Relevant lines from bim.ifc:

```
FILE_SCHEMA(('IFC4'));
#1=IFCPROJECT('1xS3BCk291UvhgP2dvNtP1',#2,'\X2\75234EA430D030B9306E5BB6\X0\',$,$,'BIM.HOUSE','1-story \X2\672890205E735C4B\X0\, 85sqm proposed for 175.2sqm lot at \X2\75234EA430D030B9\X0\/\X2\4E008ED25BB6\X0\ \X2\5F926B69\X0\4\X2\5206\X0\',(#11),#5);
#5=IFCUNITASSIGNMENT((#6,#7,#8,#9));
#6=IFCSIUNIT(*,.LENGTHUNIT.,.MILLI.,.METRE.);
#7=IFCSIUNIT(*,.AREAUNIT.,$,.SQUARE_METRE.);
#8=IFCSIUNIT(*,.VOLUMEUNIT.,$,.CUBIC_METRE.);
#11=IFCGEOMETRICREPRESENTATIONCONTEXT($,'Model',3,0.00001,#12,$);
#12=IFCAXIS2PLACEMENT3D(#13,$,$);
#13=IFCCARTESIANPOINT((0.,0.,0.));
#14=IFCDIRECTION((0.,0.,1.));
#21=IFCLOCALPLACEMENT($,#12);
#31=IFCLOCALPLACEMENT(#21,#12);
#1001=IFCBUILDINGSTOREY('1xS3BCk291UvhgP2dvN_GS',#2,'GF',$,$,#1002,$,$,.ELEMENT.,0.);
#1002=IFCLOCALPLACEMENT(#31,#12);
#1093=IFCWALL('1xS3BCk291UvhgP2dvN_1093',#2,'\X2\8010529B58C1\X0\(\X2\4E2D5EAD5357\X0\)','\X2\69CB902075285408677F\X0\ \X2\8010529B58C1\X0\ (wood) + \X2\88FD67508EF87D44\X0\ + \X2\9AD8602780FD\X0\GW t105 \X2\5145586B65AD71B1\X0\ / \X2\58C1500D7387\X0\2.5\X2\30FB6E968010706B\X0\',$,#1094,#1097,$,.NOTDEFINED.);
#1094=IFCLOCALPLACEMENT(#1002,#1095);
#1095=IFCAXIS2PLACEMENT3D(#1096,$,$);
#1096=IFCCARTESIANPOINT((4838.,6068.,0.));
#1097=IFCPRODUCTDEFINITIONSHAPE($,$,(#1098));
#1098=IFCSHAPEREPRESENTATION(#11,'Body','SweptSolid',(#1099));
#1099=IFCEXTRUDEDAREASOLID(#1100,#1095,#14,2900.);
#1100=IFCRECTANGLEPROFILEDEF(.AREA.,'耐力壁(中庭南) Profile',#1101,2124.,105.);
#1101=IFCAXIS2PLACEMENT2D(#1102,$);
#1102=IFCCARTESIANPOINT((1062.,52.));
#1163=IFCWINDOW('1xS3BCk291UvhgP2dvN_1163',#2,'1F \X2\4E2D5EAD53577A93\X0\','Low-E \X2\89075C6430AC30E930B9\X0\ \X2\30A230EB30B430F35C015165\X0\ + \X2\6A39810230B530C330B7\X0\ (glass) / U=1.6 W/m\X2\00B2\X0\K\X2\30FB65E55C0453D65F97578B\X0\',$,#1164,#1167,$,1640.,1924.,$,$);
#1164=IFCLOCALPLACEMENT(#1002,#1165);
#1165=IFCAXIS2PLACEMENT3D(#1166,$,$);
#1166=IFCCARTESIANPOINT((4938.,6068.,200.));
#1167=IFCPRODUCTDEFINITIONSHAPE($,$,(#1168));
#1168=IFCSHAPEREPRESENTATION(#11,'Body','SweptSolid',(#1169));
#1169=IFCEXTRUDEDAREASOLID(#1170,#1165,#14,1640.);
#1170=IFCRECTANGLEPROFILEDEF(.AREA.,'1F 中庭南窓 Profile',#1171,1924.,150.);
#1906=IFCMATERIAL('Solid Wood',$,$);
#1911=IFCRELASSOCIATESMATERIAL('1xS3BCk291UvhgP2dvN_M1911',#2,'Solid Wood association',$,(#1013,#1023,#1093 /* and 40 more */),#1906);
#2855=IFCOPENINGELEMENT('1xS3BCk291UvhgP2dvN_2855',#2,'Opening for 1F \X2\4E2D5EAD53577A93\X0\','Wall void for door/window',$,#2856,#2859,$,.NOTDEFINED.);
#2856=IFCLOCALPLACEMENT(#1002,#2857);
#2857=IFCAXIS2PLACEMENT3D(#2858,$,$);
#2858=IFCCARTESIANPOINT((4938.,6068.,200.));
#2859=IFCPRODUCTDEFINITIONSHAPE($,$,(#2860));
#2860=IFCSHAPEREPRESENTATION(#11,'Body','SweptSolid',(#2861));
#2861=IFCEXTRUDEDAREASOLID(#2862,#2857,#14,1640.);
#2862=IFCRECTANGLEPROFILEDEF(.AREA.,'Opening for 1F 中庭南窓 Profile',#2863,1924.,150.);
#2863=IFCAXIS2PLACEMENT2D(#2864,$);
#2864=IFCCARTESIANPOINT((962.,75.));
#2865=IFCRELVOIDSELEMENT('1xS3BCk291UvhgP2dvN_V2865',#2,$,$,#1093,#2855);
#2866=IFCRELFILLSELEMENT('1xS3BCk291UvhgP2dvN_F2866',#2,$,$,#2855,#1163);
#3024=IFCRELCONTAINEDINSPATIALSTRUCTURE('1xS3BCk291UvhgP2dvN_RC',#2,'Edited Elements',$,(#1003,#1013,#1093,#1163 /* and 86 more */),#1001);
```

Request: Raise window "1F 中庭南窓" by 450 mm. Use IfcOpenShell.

```python
import numpy as np
import ifcopenshell
import ifcopenshell.api.geometry
import ifcopenshell.util.placement
import ifcopenshell.util.unit

model = ifcopenshell.open("bim.ifc")
unit_scale = ifcopenshell.util.unit.calculate_unit_scale(model)

window = model.by_guid("1xS3BCk291UvhgP2dvN_1163")
opening = window.FillsVoids[0].RelatingOpeningElement
dz = 450.0

shift = np.array([0.0, 0.0, dz])
# The window is not placed relative to its opening, so move both.
for product in (opening, window):
    matrix = ifcopenshell.util.placement.get_local_placement(product.ObjectPlacement)
    matrix[:3, 3] += shift
    ifcopenshell.api.geometry.edit_object_placement(model, product=product, matrix=matrix, is_si=False)

print(f"moved by {dz * unit_scale:+.3f} m")

model.write("bim_rev.ifc")
```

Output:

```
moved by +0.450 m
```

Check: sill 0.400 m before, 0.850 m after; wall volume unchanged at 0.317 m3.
